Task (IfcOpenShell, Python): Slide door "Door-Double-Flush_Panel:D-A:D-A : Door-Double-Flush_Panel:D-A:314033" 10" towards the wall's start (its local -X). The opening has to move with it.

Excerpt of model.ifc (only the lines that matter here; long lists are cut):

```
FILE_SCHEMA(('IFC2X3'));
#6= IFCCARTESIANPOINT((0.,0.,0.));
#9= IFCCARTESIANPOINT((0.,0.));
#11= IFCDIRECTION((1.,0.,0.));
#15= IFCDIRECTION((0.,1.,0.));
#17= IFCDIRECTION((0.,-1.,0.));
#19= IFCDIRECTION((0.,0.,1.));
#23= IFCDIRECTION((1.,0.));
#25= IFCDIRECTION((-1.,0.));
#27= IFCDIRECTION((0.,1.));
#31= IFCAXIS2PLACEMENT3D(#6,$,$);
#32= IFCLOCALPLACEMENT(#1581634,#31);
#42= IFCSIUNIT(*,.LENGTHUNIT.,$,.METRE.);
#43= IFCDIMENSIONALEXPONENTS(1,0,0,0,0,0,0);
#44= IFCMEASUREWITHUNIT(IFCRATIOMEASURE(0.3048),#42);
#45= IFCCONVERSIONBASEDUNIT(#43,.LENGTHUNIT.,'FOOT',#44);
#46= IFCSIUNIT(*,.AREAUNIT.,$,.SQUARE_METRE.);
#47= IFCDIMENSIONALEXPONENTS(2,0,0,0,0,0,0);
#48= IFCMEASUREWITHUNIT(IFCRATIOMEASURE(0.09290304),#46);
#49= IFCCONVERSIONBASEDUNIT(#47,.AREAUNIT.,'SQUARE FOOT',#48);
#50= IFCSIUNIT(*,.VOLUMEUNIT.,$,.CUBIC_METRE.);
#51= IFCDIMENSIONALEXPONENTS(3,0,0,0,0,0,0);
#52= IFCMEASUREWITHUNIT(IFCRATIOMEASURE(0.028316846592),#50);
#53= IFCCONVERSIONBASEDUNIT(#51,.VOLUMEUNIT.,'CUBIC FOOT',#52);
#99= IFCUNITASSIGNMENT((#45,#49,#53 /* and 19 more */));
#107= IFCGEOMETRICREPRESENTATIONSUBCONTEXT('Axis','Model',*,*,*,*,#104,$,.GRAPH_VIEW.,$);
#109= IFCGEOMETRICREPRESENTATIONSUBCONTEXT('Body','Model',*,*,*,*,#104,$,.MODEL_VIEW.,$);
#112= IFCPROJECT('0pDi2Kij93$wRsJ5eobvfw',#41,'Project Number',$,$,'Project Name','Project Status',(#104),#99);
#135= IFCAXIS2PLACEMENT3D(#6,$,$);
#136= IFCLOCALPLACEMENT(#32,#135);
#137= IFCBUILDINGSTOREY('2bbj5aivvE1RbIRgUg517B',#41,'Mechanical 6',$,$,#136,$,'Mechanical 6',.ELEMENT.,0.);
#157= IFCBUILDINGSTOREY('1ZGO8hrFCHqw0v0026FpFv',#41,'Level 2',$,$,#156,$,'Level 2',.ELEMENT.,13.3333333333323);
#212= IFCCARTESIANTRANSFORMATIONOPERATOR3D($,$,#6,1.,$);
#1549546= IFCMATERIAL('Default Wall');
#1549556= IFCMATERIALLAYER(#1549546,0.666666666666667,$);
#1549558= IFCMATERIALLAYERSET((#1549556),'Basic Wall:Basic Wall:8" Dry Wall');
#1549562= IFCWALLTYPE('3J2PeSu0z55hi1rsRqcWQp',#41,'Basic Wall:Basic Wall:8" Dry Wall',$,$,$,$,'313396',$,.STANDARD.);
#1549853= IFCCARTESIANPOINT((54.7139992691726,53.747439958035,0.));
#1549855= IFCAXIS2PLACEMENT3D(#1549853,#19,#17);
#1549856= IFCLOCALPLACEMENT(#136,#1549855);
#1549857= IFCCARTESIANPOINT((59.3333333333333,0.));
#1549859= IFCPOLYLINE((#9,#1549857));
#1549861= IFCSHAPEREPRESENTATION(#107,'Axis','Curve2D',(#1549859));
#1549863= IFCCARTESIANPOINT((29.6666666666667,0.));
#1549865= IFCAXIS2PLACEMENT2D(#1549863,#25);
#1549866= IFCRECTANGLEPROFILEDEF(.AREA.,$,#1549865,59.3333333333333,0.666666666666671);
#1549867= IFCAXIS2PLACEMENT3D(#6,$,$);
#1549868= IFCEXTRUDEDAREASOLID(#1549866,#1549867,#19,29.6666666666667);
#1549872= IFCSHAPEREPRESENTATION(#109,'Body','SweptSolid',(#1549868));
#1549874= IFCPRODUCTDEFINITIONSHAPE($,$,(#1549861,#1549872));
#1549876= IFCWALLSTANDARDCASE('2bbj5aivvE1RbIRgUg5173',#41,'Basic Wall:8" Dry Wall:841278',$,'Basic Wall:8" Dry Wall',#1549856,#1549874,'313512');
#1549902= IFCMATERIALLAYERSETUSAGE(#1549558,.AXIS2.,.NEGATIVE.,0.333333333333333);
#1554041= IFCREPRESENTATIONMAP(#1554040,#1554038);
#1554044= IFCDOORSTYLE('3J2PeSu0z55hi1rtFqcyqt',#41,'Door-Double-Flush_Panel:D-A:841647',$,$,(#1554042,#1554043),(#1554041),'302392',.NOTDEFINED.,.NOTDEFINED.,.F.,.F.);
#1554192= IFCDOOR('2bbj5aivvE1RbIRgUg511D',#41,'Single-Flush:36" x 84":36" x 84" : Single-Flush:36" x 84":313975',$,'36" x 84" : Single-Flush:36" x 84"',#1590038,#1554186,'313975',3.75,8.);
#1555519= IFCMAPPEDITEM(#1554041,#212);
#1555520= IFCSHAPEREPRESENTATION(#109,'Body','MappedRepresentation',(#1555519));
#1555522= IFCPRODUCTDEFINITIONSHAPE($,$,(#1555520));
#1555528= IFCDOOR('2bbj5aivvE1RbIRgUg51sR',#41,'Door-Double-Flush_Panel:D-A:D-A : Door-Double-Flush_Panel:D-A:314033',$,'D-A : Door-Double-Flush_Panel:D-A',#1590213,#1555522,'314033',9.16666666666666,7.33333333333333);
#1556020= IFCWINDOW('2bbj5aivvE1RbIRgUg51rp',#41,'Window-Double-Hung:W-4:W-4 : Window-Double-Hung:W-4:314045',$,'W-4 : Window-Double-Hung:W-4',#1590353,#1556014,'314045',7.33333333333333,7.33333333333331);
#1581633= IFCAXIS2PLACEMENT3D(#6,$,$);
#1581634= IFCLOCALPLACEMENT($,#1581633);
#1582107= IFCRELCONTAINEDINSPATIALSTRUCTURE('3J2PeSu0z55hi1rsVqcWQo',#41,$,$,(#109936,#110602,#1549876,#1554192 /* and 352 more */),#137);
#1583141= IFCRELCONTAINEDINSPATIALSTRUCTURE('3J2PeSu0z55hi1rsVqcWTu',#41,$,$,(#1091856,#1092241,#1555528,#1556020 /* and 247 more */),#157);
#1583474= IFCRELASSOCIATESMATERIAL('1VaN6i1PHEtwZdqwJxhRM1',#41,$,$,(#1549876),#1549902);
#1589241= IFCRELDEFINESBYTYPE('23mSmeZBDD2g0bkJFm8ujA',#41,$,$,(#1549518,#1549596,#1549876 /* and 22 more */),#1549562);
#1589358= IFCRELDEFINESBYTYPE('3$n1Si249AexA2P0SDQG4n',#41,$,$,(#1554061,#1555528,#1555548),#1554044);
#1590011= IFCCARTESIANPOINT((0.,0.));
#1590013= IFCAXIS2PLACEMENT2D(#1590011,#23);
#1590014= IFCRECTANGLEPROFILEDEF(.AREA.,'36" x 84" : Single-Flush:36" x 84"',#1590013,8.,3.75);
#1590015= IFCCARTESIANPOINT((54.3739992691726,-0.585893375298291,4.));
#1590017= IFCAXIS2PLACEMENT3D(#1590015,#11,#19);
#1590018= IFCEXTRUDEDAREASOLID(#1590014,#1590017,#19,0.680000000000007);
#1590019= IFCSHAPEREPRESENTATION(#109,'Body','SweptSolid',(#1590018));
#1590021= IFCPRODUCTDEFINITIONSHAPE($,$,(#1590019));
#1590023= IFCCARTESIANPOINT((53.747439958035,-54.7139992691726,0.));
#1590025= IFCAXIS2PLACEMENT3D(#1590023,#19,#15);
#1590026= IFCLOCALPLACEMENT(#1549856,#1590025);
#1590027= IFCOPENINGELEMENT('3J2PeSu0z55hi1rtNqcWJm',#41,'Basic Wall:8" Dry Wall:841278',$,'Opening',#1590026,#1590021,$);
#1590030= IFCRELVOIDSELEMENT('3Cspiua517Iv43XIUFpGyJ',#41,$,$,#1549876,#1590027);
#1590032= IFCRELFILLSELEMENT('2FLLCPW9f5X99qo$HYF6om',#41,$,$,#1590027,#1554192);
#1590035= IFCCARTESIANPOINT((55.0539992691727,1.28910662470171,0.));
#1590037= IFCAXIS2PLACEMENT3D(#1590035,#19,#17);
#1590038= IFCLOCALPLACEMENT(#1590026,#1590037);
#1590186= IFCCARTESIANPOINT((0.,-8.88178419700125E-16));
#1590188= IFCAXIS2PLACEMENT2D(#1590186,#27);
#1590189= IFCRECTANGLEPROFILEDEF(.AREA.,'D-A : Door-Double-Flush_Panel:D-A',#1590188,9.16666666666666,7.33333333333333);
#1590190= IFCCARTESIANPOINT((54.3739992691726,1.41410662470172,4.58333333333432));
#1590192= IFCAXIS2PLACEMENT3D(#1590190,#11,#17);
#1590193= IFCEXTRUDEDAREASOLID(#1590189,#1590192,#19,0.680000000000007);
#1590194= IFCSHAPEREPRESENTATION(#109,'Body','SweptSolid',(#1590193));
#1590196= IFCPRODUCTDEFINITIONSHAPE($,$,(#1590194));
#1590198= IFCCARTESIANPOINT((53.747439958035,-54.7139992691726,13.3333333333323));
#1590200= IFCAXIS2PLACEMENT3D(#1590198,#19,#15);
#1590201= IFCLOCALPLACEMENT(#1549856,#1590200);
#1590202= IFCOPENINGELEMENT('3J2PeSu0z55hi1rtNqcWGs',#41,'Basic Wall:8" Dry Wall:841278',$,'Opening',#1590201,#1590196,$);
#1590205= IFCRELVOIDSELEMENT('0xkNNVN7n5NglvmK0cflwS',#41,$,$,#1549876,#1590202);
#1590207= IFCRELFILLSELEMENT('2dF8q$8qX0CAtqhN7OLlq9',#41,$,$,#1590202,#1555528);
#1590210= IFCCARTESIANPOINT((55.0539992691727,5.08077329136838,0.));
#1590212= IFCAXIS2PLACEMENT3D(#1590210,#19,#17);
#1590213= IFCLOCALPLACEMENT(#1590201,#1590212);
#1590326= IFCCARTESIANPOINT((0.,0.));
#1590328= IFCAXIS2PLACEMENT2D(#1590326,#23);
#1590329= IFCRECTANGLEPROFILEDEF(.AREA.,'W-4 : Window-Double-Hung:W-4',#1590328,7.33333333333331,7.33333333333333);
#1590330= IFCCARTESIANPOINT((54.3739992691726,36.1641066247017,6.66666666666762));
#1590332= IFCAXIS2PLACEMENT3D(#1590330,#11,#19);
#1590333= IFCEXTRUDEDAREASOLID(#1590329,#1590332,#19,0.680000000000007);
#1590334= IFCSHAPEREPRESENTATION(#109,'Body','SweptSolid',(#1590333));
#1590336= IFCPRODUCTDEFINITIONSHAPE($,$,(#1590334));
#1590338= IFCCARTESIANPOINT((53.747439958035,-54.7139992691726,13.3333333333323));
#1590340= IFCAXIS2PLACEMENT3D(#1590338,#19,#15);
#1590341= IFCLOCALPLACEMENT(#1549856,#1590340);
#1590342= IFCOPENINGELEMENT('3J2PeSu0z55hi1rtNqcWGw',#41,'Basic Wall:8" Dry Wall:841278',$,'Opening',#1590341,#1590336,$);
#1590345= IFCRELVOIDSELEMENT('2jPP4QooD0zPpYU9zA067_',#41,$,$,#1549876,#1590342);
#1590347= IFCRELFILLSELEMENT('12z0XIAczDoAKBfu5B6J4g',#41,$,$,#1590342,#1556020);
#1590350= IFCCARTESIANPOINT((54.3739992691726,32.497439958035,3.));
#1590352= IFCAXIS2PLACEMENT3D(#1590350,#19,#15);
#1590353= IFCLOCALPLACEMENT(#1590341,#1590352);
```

```python
import ifcopenshell
import ifcopenshell.api.geometry
import ifcopenshell.util.placement
import ifcopenshell.util.unit

model = ifcopenshell.open("model.ifc")
unit_scale = ifcopenshell.util.unit.calculate_unit_scale(model)

door = model.by_guid("2bbj5aivvE1RbIRgUg51sR")
opening = door.FillsVoids[0].RelatingOpeningElement
wall = opening.VoidsElements[0].RelatingBuildingElement

wall_matrix = ifcopenshell.util.placement.get_local_placement(wall.ObjectPlacement)
shift = wall_matrix[:3, 0] * -10 * 0.0254 / unit_scale
before = ifcopenshell.util.placement.get_local_placement(door.ObjectPlacement)[:3, 3].copy()

# The door is placed relative to its opening, so it follows when the opening moves.
matrix = ifcopenshell.util.placement.get_local_placement(opening.ObjectPlacement)
matrix[:3, 3] += shift
ifcopenshell.api.geometry.edit_object_placement(
    model, product=opening, matrix=matrix, is_si=False, should_transform_children=True
)

after = ifcopenshell.util.placement.get_local_placement(door.ObjectPlacement)[:3, 3]
print("door moved by", (after - before).round(3) + 0.0)

model.write("model_v2.ifc")
```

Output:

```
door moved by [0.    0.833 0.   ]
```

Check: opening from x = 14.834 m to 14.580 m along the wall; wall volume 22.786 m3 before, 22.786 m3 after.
